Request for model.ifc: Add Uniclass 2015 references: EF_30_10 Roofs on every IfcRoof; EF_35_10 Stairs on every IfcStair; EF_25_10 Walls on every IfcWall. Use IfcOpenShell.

First a look at what the model holds.

```python
import ifcopenshell

model = ifcopenshell.open("model.ifc")
print(model.schema)
print("classifications:", [c.Name for c in model.by_type("IfcClassification")])
for ifc_class in ("IfcDoor", "IfcRoof", "IfcStair", "IfcWall", "IfcWindow"):
    print(ifc_class, len(model.by_type(ifc_class)))
```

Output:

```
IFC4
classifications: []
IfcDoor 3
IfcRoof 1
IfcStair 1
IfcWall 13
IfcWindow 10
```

```python
import ifcopenshell
import ifcopenshell.api.classification

model = ifcopenshell.open("model.ifc")

system = ifcopenshell.api.classification.add_classification(model, classification="Uniclass 2015")

codes = {
    "IfcRoof": ("EF_30_10", "Roofs"),
    "IfcStair": ("EF_35_10", "Stairs"),
    "IfcWall": ("EF_25_10", "Walls"),
}
for ifc_class, (code, name) in codes.items():
    products = model.by_type(ifc_class)
    ifcopenshell.api.classification.add_reference(
        model, products=products, classification=system, identification=code, name=name
    )
    print(code, len(products))

model.write("model_updated.ifc")
```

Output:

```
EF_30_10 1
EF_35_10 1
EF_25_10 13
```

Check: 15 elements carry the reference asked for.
